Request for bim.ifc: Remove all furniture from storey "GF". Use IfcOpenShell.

First a look at what the model holds.

```python
import ifcopenshell
import ifcopenshell.util.element

model = ifcopenshell.open("bim.ifc")
print(model.schema)
storey = next(s for s in model.by_type("IfcBuildingStorey") if s.Name == "GF")
furniture = [e for e in ifcopenshell.util.element.get_decomposition(storey) if e.is_a("IfcFurnishingElement")]
seen = {}
for e in furniture:
    element_type = ifcopenshell.util.element.get_type(e)
    name = element_type.Name if element_type not in (None, e) else None
    seen[name] = seen.get(name, 0) + 1
for name, count in sorted(seen.items(), key=str):
    print(count, "x", name)
```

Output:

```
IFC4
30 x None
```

```python
import ifcopenshell
import ifcopenshell.api.root
import ifcopenshell.util.element

model = ifcopenshell.open("bim.ifc")

storey = next(s for s in model.by_type("IfcBuildingStorey") if s.Name == "GF")
furniture = [e for e in ifcopenshell.util.element.get_decomposition(storey) if e.is_a("IfcFurnishingElement")]

for e in furniture:
    ifcopenshell.api.root.remove_product(model, product=e)
print(len(furniture), "removed")

model.write("bim-out.ifc")
```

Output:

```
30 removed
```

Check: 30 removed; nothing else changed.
